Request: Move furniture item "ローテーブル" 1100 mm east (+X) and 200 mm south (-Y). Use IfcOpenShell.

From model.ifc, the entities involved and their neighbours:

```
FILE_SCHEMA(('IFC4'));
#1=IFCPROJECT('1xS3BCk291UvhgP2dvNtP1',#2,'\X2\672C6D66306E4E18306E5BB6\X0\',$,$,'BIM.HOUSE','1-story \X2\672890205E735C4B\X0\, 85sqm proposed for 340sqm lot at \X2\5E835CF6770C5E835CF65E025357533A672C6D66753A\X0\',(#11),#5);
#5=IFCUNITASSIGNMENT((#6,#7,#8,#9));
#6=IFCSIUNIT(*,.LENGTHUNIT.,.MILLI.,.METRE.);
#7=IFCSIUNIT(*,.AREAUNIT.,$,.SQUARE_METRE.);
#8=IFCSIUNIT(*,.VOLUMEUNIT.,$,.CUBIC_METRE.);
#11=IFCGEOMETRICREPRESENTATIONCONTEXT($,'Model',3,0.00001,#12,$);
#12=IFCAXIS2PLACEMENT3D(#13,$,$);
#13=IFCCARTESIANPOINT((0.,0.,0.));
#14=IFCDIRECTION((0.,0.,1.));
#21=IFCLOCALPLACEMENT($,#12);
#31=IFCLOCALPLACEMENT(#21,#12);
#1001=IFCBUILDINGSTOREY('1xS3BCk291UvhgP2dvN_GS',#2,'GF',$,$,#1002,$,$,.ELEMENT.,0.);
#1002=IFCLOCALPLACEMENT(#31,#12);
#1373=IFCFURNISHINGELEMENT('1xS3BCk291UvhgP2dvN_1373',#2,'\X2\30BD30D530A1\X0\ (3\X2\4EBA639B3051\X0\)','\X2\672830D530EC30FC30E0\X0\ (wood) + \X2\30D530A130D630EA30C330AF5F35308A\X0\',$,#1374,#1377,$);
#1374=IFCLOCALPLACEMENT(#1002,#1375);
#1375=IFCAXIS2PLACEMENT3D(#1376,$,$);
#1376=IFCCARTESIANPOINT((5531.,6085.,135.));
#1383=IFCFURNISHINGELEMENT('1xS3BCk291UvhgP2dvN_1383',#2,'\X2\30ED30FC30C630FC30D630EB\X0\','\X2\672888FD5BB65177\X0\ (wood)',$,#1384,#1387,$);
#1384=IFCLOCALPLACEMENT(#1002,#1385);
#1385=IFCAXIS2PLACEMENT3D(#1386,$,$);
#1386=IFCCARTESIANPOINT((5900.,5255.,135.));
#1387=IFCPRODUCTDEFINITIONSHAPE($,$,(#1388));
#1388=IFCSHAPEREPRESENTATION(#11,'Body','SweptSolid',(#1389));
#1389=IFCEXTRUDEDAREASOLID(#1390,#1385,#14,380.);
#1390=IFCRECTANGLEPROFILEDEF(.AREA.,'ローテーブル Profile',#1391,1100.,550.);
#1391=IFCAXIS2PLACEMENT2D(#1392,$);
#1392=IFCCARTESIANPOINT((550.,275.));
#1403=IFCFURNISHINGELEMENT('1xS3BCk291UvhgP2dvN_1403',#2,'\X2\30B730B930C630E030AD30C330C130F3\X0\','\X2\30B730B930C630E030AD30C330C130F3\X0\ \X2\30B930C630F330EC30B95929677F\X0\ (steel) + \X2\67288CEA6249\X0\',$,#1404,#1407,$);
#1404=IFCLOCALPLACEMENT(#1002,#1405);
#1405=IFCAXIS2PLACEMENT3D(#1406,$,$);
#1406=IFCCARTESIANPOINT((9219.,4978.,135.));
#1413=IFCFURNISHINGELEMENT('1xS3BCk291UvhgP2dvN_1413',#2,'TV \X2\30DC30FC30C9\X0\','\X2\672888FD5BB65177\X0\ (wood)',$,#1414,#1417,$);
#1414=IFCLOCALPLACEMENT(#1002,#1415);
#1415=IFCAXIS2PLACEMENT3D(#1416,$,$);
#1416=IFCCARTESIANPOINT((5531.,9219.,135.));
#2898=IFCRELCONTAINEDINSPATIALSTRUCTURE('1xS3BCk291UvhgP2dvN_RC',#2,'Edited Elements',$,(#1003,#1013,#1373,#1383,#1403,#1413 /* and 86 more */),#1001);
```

```python
import ifcopenshell
import ifcopenshell.api.geometry
import ifcopenshell.util.placement

model = ifcopenshell.open("model.ifc")

item = model.by_id(1383)
matrix = ifcopenshell.util.placement.get_local_placement(item.ObjectPlacement)
matrix[0, 3] += 1100.0
matrix[1, 3] -= 200.0
ifcopenshell.api.geometry.edit_object_placement(model, product=item, matrix=matrix, is_si=False)

print(ifcopenshell.util.placement.get_local_placement(item.ObjectPlacement).round(3) + 0.0)

model.write("model_rev.ifc")
```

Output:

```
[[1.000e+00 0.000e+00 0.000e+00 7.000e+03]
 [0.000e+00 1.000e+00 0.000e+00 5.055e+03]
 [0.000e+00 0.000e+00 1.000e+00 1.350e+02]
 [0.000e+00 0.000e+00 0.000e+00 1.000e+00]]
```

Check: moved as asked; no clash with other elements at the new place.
